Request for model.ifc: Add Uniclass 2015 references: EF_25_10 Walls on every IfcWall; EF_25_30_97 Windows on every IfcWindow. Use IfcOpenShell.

First a look at what the model holds.

```python
import ifcopenshell

model = ifcopenshell.open("model.ifc")
print(model.schema)
print("classifications:", [c.Name for c in model.by_type("IfcClassification")])
for ifc_class in ("IfcDoor", "IfcRoof", "IfcStair", "IfcWall", "IfcWindow"):
    print(ifc_class, len(model.by_type(ifc_class)))
```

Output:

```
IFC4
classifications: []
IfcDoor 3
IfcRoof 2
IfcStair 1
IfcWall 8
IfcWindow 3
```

```python
import ifcopenshell
import ifcopenshell.api.classification

model = ifcopenshell.open("model.ifc")

system = ifcopenshell.api.classification.add_classification(model, classification="Uniclass 2015")

codes = {
    "IfcWall": ("EF_25_10", "Walls"),
    "IfcWindow": ("EF_25_30_97", "Windows"),
}
for ifc_class, (code, name) in codes.items():
    products = model.by_type(ifc_class)
    ifcopenshell.api.classification.add_reference(
        model, products=products, classification=system, identification=code, name=name
    )
    print(code, len(products))

model.write("model_edited.ifc")
```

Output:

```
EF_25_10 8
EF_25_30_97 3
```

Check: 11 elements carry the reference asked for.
